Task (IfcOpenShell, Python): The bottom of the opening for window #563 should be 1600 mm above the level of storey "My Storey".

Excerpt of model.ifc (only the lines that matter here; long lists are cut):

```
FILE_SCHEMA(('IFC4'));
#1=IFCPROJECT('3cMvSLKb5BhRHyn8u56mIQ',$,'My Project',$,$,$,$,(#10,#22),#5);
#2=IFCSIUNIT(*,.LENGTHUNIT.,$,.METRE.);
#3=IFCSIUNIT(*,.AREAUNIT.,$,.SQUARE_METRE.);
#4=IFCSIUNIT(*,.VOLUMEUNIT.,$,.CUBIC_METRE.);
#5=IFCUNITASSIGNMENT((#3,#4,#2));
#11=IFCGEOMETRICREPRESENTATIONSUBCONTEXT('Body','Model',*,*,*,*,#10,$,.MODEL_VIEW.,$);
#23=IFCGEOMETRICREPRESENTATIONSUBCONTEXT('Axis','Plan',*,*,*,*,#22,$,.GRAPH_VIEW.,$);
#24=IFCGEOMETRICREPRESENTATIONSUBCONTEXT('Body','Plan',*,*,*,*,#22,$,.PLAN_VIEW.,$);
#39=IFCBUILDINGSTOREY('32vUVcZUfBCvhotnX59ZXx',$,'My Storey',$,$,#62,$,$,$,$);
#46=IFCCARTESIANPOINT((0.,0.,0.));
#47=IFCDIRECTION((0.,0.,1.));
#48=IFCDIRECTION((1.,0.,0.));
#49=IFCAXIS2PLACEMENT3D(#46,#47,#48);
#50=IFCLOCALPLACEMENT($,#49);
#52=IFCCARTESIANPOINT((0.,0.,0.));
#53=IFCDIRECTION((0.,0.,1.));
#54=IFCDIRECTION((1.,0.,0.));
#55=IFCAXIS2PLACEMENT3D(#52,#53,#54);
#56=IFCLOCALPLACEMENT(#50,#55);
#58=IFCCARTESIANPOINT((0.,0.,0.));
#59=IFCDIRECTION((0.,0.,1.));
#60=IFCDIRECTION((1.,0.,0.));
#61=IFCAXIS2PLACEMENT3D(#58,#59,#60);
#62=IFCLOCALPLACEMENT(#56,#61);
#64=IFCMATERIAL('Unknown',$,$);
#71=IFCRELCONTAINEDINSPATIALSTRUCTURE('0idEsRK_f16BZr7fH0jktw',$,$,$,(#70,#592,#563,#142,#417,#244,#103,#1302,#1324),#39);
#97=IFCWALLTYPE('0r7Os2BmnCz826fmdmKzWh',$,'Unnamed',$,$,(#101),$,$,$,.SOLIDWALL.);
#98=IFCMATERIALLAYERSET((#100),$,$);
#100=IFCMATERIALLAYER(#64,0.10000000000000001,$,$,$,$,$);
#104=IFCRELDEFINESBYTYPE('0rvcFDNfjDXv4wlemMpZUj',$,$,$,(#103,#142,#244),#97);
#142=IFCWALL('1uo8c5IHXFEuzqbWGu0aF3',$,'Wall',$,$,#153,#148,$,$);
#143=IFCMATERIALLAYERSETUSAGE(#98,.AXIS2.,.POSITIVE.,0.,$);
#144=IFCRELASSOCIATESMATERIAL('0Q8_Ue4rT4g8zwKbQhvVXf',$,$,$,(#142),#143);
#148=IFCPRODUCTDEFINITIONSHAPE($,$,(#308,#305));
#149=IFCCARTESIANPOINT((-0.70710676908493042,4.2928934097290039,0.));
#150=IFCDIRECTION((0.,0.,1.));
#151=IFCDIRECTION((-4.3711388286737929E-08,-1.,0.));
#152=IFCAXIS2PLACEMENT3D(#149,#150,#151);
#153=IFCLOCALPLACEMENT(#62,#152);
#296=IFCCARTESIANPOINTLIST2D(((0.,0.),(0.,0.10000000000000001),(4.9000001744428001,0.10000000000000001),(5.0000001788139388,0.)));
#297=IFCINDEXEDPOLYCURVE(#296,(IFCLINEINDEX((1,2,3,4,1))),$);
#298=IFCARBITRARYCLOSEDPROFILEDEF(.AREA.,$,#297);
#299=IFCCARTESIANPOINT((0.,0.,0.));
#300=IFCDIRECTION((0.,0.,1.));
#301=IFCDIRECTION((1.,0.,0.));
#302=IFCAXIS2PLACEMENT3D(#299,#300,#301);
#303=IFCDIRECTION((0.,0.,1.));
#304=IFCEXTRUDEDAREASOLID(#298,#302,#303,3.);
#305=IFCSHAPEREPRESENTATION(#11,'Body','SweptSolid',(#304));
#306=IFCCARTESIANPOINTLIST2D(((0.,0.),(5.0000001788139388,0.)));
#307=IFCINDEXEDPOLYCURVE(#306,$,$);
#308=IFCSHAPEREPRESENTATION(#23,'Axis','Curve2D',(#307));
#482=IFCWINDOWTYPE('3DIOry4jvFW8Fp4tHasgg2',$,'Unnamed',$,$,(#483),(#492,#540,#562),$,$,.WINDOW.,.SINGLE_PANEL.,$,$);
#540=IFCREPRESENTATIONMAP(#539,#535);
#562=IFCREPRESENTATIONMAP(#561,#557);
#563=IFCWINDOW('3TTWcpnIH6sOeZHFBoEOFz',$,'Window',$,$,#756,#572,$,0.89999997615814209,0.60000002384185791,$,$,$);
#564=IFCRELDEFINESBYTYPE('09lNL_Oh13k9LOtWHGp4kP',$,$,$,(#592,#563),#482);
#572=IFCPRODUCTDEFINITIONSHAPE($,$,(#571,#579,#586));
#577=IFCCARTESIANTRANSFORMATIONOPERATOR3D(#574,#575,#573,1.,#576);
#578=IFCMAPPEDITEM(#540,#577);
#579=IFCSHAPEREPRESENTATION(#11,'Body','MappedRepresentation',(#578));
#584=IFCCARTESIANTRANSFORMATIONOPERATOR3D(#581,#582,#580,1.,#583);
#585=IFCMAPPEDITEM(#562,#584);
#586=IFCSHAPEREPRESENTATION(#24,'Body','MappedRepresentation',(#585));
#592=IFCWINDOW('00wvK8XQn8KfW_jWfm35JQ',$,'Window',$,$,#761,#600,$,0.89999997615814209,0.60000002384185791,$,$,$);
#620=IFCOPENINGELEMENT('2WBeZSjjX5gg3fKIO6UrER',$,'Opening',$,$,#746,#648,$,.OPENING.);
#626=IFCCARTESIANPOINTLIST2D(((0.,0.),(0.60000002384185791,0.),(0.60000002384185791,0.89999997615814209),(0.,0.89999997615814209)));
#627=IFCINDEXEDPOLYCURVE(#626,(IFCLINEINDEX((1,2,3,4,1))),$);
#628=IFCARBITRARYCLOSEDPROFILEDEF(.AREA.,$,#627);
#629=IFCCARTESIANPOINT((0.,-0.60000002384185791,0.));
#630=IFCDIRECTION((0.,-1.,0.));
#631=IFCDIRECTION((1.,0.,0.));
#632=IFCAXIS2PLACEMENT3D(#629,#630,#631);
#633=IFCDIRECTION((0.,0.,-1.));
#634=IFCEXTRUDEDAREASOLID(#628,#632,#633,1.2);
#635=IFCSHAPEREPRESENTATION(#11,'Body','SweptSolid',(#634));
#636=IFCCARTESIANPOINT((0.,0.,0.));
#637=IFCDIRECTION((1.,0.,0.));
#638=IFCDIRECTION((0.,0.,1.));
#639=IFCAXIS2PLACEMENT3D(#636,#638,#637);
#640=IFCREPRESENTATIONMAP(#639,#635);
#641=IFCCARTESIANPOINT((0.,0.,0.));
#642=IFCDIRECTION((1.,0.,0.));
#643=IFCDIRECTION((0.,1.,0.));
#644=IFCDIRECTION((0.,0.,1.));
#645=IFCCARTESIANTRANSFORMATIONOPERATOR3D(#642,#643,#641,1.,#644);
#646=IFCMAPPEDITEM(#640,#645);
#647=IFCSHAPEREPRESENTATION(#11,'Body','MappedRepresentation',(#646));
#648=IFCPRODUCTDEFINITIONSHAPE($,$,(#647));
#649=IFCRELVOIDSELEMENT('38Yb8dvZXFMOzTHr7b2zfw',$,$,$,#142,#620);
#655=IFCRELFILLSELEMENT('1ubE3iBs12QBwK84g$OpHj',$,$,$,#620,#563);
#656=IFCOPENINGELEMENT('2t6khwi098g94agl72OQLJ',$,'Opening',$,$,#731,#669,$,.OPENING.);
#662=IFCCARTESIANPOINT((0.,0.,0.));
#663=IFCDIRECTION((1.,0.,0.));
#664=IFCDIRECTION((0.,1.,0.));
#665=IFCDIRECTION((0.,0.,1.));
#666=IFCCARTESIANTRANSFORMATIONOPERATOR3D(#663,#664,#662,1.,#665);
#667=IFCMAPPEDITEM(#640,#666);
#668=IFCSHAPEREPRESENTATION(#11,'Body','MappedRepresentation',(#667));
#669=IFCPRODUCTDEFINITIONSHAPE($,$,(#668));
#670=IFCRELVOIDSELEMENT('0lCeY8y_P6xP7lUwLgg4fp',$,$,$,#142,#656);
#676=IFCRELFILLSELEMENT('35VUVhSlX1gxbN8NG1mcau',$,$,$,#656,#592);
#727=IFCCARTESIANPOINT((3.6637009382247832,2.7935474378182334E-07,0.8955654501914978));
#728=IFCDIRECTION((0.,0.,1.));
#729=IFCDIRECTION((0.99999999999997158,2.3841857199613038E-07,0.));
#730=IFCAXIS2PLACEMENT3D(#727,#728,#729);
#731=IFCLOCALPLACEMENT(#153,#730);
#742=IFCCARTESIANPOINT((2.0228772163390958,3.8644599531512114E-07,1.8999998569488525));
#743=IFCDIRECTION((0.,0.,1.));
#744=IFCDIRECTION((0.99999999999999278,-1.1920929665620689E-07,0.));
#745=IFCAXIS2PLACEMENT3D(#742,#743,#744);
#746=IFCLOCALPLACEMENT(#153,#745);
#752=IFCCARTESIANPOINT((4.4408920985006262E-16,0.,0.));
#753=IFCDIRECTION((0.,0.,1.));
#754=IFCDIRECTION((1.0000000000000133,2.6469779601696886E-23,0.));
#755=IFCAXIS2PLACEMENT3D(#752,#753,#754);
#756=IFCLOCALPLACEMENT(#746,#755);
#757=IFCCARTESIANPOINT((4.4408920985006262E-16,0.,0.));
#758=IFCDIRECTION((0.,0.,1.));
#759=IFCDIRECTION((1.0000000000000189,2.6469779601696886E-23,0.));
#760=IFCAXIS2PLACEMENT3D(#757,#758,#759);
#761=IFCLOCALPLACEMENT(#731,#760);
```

```python
import numpy as np
import ifcopenshell
import ifcopenshell.api.geometry
import ifcopenshell.geom
import ifcopenshell.util.element
import ifcopenshell.util.placement
import ifcopenshell.util.shape
import ifcopenshell.util.unit

model = ifcopenshell.open("model.ifc")
unit_scale = ifcopenshell.util.unit.calculate_unit_scale(model)

window = model.by_guid("3TTWcpnIH6sOeZHFBoEOFz")
opening = window.FillsVoids[0].RelatingOpeningElement
storey = ifcopenshell.util.element.get_container(window, ifc_class="IfcBuildingStorey")
level = ifcopenshell.util.placement.get_local_placement(storey.ObjectPlacement)[2, 3]

# The opening's origin need not be at the sill, so measure its lowest point.
shape = ifcopenshell.geom.create_shape(ifcopenshell.geom.settings(), opening)
bottom = ifcopenshell.util.shape.get_shape_bottom_elevation(shape, shape.geometry) / unit_scale
dz = level + 1.6 - bottom

shift = np.array([0.0, 0.0, dz])
# The window is placed relative to its opening, so it follows when the opening moves.
matrix = ifcopenshell.util.placement.get_local_placement(opening.ObjectPlacement)
matrix[:3, 3] += shift
ifcopenshell.api.geometry.edit_object_placement(
    model, product=opening, matrix=matrix, is_si=False, should_transform_children=True
)

print(f"moved by {dz * unit_scale:+.3f} m")

model.write("model_updated.ifc")
```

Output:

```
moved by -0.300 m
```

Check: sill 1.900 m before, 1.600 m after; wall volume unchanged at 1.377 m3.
